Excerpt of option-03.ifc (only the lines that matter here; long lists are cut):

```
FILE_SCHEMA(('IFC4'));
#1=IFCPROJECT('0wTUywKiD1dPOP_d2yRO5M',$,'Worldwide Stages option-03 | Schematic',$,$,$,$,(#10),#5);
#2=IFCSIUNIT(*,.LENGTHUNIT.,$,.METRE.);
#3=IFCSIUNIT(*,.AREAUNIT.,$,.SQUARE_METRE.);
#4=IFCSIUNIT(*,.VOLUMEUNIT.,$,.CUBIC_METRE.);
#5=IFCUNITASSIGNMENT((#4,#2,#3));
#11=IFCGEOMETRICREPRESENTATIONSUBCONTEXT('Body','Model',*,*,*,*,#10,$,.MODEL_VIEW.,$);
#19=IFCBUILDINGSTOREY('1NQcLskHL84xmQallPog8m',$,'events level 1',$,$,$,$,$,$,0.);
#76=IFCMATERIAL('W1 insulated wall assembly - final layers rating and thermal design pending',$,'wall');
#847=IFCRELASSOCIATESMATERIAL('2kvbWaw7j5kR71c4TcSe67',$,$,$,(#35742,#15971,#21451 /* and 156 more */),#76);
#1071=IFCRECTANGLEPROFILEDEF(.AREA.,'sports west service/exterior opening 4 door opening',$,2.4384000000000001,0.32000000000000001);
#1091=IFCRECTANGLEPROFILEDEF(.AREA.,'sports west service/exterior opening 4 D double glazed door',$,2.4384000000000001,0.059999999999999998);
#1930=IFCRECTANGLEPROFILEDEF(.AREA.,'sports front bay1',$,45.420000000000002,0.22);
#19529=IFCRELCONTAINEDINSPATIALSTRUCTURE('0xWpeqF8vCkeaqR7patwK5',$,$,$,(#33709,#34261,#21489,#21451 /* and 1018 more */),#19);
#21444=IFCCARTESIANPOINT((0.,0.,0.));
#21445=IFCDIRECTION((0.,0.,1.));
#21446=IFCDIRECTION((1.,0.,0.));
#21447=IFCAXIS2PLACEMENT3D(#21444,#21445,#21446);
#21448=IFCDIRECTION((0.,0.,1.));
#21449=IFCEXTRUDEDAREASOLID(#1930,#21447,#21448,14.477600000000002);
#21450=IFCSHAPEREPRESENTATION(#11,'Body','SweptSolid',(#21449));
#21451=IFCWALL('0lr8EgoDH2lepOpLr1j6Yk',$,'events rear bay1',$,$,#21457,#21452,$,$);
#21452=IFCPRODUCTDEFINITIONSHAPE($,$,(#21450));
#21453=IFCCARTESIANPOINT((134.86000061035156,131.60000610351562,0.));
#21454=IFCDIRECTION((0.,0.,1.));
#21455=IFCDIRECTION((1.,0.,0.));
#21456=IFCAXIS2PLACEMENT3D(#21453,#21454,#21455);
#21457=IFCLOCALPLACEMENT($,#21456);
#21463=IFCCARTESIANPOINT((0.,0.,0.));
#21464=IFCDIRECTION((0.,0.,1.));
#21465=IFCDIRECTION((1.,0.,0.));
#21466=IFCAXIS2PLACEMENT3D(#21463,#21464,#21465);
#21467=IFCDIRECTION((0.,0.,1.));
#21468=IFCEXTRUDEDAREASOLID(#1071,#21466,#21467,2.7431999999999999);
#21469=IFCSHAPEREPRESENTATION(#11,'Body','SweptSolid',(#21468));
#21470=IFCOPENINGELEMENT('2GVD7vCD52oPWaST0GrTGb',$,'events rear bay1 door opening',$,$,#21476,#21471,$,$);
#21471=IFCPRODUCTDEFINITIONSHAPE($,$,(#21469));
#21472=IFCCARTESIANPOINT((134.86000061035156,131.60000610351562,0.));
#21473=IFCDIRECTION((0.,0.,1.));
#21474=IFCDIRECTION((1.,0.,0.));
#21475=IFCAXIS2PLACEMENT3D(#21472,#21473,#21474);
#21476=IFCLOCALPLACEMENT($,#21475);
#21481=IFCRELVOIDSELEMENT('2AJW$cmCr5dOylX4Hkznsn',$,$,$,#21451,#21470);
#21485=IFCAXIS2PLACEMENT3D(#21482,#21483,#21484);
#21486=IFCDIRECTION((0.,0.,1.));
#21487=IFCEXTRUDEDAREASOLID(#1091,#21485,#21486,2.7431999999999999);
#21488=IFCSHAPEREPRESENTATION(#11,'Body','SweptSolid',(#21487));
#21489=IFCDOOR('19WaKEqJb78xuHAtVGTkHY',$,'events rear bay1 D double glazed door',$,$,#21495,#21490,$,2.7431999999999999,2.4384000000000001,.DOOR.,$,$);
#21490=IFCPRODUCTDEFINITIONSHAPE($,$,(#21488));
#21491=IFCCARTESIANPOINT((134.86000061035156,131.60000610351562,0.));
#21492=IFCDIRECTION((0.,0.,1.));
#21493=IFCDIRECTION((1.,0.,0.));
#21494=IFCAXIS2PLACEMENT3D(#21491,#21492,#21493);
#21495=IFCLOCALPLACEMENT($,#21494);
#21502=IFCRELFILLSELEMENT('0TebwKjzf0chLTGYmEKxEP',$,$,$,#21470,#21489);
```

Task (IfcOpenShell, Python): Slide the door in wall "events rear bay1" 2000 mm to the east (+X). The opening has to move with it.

```python
import ifcopenshell
import ifcopenshell.api.geometry
import ifcopenshell.util.placement
import ifcopenshell.util.unit

model = ifcopenshell.open("option-03.ifc")
unit_scale = ifcopenshell.util.unit.calculate_unit_scale(model)

door = model.by_guid("19WaKEqJb78xuHAtVGTkHY")
opening = door.FillsVoids[0].RelatingOpeningElement
wall = opening.VoidsElements[0].RelatingBuildingElement

wall_matrix = ifcopenshell.util.placement.get_local_placement(wall.ObjectPlacement)
shift = wall_matrix[:3, 0] * 2 / unit_scale
before = ifcopenshell.util.placement.get_local_placement(door.ObjectPlacement)[:3, 3].copy()

# The door is not placed relative to its opening, so move both.
for product in (opening, door):
    matrix = ifcopenshell.util.placement.get_local_placement(product.ObjectPlacement)
    matrix[:3, 3] += shift
    ifcopenshell.api.geometry.edit_object_placement(model, product=product, matrix=matrix, is_si=False)

after = ifcopenshell.util.placement.get_local_placement(door.ObjectPlacement)[:3, 3]
print("door moved by", (after - before).round(3) + 0.0)

model.write("option-03_edited.ifc")
```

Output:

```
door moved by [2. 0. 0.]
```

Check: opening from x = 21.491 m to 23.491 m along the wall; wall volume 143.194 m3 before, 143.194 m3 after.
